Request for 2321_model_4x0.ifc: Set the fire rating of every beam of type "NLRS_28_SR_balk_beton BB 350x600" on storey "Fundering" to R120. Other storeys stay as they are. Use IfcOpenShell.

First a look at what the model holds.

```python
import ifcopenshell
import ifcopenshell.util.element

model = ifcopenshell.open("2321_model_4x0.ifc")
print(model.schema)
storey = next(s for s in model.by_type("IfcBuildingStorey") if s.Name == "Fundering")
beams = [e for e in ifcopenshell.util.element.get_decomposition(storey) if e.is_a("IfcBeam")]
seen = {}
for e in beams:
    element_type = ifcopenshell.util.element.get_type(e)
    key = (element_type.Name if element_type != e and element_type else None, ifcopenshell.util.element.get_pset(e, "Pset_BeamCommon", "FireRating"))
    seen[key] = seen.get(key, 0) + 1
for (name, value), count in sorted(seen.items(), key=str):
    print(count, "x", name, "|", value)
```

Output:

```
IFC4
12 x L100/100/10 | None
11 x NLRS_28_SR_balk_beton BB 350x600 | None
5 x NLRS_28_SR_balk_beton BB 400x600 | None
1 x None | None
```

```python
import ifcopenshell
import ifcopenshell.api.pset
import ifcopenshell.util.element

model = ifcopenshell.open("2321_model_4x0.ifc")

storey = next(s for s in model.by_type("IfcBuildingStorey") if s.Name == "Fundering")
beams = [e for e in ifcopenshell.util.element.get_decomposition(storey) if e.is_a("IfcBeam")]

count = 0
for e in beams:
    element_type = ifcopenshell.util.element.get_type(e)
    if element_type in (None, e) or element_type.Name != "NLRS_28_SR_balk_beton BB 350x600":
        continue
    # add_pset returns the element's existing set when there is one.
    pset = ifcopenshell.api.pset.add_pset(model, product=e, name="Pset_BeamCommon")
    ifcopenshell.api.pset.edit_pset(model, pset=pset, properties={"FireRating": "R120"})
    count += 1

print(count, "beams updated")

model.write("2321_model_4x0-out.ifc")
```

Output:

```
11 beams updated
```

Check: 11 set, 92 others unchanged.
